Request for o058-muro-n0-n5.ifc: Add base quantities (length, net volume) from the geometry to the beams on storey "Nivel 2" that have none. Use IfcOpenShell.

First a look at what the model holds.

```python
import ifcopenshell
import ifcopenshell.util.element
import ifcopenshell.util.unit

model = ifcopenshell.open("o058-muro-n0-n5.ifc")
print(model.schema)
for unit_type in ("LENGTHUNIT", "AREAUNIT", "VOLUMEUNIT"):
    print(unit_type, ifcopenshell.util.unit.calculate_unit_scale(model, unit_type))
storey = next(s for s in model.by_type("IfcBuildingStorey") if s.Name == "Nivel 2")
beams = [e for e in ifcopenshell.util.element.get_decomposition(storey) if e.is_a("IfcBeam")]
for e in sorted(beams, key=lambda e: e.id()):
    print(e.id(), e.is_a(), e.Name, list(ifcopenshell.util.element.get_psets(e, qtos_only=True)), sep=" | ")
```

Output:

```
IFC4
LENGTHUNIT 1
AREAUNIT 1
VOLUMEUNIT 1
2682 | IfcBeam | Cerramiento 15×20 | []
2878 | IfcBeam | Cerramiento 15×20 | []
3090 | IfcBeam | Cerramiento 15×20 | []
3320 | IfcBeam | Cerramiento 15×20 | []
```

```python
import ifcopenshell
import ifcopenshell.api.pset
import ifcopenshell.geom
import ifcopenshell.util.element
import ifcopenshell.util.shape
import ifcopenshell.util.unit

model = ifcopenshell.open("o058-muro-n0-n5.ifc")
unit_scale = ifcopenshell.util.unit.calculate_unit_scale(model)
volume_scale = ifcopenshell.util.unit.calculate_unit_scale(model, "VOLUMEUNIT")
settings = ifcopenshell.geom.settings()

storey = next(s for s in model.by_type("IfcBuildingStorey") if s.Name == "Nivel 2")
beams = [e for e in ifcopenshell.util.element.get_decomposition(storey) if e.is_a("IfcBeam")]

for e in sorted(beams, key=lambda e: e.id()):
    if ifcopenshell.util.element.get_psets(e, qtos_only=True, should_inherit=False):
        continue
    # Geometry comes back in metres, in the element's own axes.
    shape = ifcopenshell.geom.create_shape(settings, e)
    values = {
        "Length": ifcopenshell.util.shape.get_max_xyz(shape.geometry) / unit_scale,
        "NetVolume": ifcopenshell.util.shape.get_volume(shape.geometry) / volume_scale,
    }
    qto = ifcopenshell.api.pset.add_qto(model, product=e, name="Qto_BeamBaseQuantities")
    ifcopenshell.api.pset.edit_qto(model, qto=qto, properties=values)
    print(e.id(), {k: round(v, 3) for k, v in values.items()})

model.write("o058-muro-n0-n5_edited.ifc")
```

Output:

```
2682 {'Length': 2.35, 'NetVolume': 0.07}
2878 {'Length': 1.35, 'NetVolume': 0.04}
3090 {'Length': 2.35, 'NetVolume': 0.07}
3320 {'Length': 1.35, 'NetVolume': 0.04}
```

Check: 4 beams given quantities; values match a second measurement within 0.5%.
